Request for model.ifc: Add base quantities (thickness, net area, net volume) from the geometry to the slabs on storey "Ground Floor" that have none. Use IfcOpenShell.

First a look at what the model holds.

```python
import ifcopenshell
import ifcopenshell.util.element
import ifcopenshell.util.unit

model = ifcopenshell.open("model.ifc")
print(model.schema)
for unit_type in ("LENGTHUNIT", "AREAUNIT", "VOLUMEUNIT"):
    print(unit_type, ifcopenshell.util.unit.calculate_unit_scale(model, unit_type))
storey = next(s for s in model.by_type("IfcBuildingStorey") if s.Name == "Ground Floor")
slabs = [e for e in ifcopenshell.util.element.get_decomposition(storey) if e.is_a("IfcSlab")]
for e in sorted(slabs, key=lambda e: e.id()):
    print(e.id(), e.is_a(), e.Name, list(ifcopenshell.util.element.get_psets(e, qtos_only=True)), sep=" | ")
```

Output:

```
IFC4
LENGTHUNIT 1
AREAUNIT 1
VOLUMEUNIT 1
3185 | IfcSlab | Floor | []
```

```python
import ifcopenshell
import ifcopenshell.api.pset
import ifcopenshell.geom
import ifcopenshell.util.element
import ifcopenshell.util.shape
import ifcopenshell.util.unit

model = ifcopenshell.open("model.ifc")
unit_scale = ifcopenshell.util.unit.calculate_unit_scale(model)
area_scale = ifcopenshell.util.unit.calculate_unit_scale(model, "AREAUNIT")
volume_scale = ifcopenshell.util.unit.calculate_unit_scale(model, "VOLUMEUNIT")
settings = ifcopenshell.geom.settings()

storey = next(s for s in model.by_type("IfcBuildingStorey") if s.Name == "Ground Floor")
slabs = [e for e in ifcopenshell.util.element.get_decomposition(storey) if e.is_a("IfcSlab")]

for e in sorted(slabs, key=lambda e: e.id()):
    if ifcopenshell.util.element.get_psets(e, qtos_only=True, should_inherit=False):
        continue
    # Geometry comes back in metres, in the element's own axes.
    shape = ifcopenshell.geom.create_shape(settings, e)
    values = {
        "Width": ifcopenshell.util.shape.get_z(shape.geometry) / unit_scale,
        "NetArea": ifcopenshell.util.shape.get_footprint_area(shape.geometry) / area_scale,
        "NetVolume": ifcopenshell.util.shape.get_volume(shape.geometry) / volume_scale,
    }
    qto = ifcopenshell.api.pset.add_qto(model, product=e, name="Qto_SlabBaseQuantities")
    ifcopenshell.api.pset.edit_qto(model, qto=qto, properties=values)
    print(e.id(), {k: round(v, 3) for k, v in values.items()})

model.write("model_updated.ifc")
```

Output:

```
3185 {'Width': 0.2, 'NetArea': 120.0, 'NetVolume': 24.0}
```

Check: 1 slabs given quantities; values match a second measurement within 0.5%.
